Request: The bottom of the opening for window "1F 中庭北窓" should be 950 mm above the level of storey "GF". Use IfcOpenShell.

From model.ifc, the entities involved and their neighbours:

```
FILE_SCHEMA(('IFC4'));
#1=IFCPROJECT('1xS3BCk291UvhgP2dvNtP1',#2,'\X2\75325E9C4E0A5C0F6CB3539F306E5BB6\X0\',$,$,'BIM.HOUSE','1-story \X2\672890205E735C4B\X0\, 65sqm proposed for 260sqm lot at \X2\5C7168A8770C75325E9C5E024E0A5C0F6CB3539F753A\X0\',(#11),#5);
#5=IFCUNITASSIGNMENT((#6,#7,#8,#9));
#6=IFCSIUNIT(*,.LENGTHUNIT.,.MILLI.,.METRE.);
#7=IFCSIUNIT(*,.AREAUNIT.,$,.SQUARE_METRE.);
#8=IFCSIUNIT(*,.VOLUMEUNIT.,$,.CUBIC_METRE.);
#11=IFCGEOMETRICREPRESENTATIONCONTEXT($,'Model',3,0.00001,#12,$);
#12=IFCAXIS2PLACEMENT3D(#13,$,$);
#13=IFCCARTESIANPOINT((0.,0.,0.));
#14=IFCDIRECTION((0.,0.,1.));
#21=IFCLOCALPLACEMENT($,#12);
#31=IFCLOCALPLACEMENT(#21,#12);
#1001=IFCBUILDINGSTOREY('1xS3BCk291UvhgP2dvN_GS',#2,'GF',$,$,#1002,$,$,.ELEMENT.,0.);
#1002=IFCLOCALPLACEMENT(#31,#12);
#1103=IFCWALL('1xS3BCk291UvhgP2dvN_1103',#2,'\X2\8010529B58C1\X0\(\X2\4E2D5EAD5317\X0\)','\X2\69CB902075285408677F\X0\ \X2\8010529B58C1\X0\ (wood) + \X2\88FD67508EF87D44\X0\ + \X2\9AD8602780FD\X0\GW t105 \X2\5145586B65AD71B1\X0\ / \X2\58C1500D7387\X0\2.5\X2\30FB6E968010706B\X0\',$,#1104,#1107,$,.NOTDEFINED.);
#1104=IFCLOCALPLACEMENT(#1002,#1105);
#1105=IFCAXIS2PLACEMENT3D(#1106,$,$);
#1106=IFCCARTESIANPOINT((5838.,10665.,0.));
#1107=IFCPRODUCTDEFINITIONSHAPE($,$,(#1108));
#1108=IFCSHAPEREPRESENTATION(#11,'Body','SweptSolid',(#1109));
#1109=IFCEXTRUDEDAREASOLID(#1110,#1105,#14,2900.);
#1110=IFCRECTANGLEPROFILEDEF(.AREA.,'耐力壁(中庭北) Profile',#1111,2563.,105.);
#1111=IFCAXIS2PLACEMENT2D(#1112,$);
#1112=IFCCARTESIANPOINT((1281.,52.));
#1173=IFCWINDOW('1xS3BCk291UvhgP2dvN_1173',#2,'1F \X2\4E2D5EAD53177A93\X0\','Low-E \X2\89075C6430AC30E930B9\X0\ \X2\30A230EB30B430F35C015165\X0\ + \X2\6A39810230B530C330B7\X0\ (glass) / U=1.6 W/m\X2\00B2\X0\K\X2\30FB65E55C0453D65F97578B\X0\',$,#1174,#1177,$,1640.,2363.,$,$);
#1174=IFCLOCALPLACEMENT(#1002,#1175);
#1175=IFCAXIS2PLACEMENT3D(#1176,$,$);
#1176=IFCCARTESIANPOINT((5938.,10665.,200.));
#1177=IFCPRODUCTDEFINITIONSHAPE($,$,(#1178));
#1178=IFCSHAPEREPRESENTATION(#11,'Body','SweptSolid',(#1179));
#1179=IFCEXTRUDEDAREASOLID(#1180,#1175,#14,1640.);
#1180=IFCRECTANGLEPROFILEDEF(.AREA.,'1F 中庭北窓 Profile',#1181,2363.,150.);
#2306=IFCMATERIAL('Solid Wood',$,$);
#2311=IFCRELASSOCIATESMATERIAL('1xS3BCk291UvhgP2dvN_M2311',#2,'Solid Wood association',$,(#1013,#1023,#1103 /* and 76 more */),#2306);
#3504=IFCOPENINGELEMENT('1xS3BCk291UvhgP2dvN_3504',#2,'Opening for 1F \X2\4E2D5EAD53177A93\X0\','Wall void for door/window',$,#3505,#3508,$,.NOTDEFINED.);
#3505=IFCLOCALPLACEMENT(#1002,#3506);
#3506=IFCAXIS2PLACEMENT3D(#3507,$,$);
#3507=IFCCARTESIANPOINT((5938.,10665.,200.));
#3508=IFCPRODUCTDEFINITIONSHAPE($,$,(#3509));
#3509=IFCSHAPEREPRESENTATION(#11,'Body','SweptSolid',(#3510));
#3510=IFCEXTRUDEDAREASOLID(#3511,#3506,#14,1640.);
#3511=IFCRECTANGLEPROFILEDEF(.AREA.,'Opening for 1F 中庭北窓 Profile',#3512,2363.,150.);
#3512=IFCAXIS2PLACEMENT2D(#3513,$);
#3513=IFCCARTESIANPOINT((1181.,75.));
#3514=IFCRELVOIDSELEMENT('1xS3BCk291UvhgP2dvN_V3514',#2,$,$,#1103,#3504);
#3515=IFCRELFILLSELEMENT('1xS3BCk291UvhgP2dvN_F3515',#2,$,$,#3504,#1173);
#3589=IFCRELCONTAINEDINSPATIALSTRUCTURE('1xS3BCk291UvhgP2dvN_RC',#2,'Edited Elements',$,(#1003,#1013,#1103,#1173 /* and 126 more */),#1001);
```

```python
import numpy as np
import ifcopenshell
import ifcopenshell.api.geometry
import ifcopenshell.geom
import ifcopenshell.util.element
import ifcopenshell.util.placement
import ifcopenshell.util.shape
import ifcopenshell.util.unit

model = ifcopenshell.open("model.ifc")
unit_scale = ifcopenshell.util.unit.calculate_unit_scale(model)

window = model.by_guid("1xS3BCk291UvhgP2dvN_1173")
opening = window.FillsVoids[0].RelatingOpeningElement
storey = ifcopenshell.util.element.get_container(window, ifc_class="IfcBuildingStorey")
level = ifcopenshell.util.placement.get_local_placement(storey.ObjectPlacement)[2, 3]

# The opening's origin need not be at the sill, so measure its lowest point.
shape = ifcopenshell.geom.create_shape(ifcopenshell.geom.settings(), opening)
bottom = ifcopenshell.util.shape.get_shape_bottom_elevation(shape, shape.geometry) / unit_scale
dz = level + 950.0 - bottom

shift = np.array([0.0, 0.0, dz])
# The window is not placed relative to its opening, so move both.
for product in (opening, window):
    matrix = ifcopenshell.util.placement.get_local_placement(product.ObjectPlacement)
    matrix[:3, 3] += shift
    ifcopenshell.api.geometry.edit_object_placement(model, product=product, matrix=matrix, is_si=False)

print(f"moved by {dz * unit_scale:+.3f} m")

model.write("model_edited.ifc")
```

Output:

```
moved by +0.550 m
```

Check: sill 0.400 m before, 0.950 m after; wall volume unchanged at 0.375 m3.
